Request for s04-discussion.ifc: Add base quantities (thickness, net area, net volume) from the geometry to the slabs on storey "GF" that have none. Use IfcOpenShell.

First a look at what the model holds.

```python
import ifcopenshell
import ifcopenshell.util.element
import ifcopenshell.util.unit

model = ifcopenshell.open("s04-discussion.ifc")
print(model.schema)
for unit_type in ("LENGTHUNIT", "AREAUNIT", "VOLUMEUNIT"):
    print(unit_type, ifcopenshell.util.unit.calculate_unit_scale(model, unit_type))
storey = next(s for s in model.by_type("IfcBuildingStorey") if s.Name == "GF")
slabs = [e for e in ifcopenshell.util.element.get_decomposition(storey) if e.is_a("IfcSlab")]
for e in sorted(slabs, key=lambda e: e.id()):
    print(e.id(), e.is_a(), e.Name, list(ifcopenshell.util.element.get_psets(e, qtos_only=True)), sep=" | ")
```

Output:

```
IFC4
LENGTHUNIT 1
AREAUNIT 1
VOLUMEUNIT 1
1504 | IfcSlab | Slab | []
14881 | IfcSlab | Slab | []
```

```python
import ifcopenshell
import ifcopenshell.api.pset
import ifcopenshell.geom
import ifcopenshell.util.element
import ifcopenshell.util.shape
import ifcopenshell.util.unit

model = ifcopenshell.open("s04-discussion.ifc")
unit_scale = ifcopenshell.util.unit.calculate_unit_scale(model)
area_scale = ifcopenshell.util.unit.calculate_unit_scale(model, "AREAUNIT")
volume_scale = ifcopenshell.util.unit.calculate_unit_scale(model, "VOLUMEUNIT")
settings = ifcopenshell.geom.settings()

storey = next(s for s in model.by_type("IfcBuildingStorey") if s.Name == "GF")
slabs = [e for e in ifcopenshell.util.element.get_decomposition(storey) if e.is_a("IfcSlab")]

for e in sorted(slabs, key=lambda e: e.id()):
    if ifcopenshell.util.element.get_psets(e, qtos_only=True, should_inherit=False):
        continue
    # Geometry comes back in metres, in the element's own axes.
    shape = ifcopenshell.geom.create_shape(settings, e)
    values = {
        "Width": ifcopenshell.util.shape.get_z(shape.geometry) / unit_scale,
        "NetArea": ifcopenshell.util.shape.get_footprint_area(shape.geometry) / area_scale,
        "NetVolume": ifcopenshell.util.shape.get_volume(shape.geometry) / volume_scale,
    }
    qto = ifcopenshell.api.pset.add_qto(model, product=e, name="Qto_SlabBaseQuantities")
    ifcopenshell.api.pset.edit_qto(model, qto=qto, properties=values)
    print(e.id(), {k: round(v, 3) for k, v in values.items()})

model.write("s04-discussion_edited.ifc")
```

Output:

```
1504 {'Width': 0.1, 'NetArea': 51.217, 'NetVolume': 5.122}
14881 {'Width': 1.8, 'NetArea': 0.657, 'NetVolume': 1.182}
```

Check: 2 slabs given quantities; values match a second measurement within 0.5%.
